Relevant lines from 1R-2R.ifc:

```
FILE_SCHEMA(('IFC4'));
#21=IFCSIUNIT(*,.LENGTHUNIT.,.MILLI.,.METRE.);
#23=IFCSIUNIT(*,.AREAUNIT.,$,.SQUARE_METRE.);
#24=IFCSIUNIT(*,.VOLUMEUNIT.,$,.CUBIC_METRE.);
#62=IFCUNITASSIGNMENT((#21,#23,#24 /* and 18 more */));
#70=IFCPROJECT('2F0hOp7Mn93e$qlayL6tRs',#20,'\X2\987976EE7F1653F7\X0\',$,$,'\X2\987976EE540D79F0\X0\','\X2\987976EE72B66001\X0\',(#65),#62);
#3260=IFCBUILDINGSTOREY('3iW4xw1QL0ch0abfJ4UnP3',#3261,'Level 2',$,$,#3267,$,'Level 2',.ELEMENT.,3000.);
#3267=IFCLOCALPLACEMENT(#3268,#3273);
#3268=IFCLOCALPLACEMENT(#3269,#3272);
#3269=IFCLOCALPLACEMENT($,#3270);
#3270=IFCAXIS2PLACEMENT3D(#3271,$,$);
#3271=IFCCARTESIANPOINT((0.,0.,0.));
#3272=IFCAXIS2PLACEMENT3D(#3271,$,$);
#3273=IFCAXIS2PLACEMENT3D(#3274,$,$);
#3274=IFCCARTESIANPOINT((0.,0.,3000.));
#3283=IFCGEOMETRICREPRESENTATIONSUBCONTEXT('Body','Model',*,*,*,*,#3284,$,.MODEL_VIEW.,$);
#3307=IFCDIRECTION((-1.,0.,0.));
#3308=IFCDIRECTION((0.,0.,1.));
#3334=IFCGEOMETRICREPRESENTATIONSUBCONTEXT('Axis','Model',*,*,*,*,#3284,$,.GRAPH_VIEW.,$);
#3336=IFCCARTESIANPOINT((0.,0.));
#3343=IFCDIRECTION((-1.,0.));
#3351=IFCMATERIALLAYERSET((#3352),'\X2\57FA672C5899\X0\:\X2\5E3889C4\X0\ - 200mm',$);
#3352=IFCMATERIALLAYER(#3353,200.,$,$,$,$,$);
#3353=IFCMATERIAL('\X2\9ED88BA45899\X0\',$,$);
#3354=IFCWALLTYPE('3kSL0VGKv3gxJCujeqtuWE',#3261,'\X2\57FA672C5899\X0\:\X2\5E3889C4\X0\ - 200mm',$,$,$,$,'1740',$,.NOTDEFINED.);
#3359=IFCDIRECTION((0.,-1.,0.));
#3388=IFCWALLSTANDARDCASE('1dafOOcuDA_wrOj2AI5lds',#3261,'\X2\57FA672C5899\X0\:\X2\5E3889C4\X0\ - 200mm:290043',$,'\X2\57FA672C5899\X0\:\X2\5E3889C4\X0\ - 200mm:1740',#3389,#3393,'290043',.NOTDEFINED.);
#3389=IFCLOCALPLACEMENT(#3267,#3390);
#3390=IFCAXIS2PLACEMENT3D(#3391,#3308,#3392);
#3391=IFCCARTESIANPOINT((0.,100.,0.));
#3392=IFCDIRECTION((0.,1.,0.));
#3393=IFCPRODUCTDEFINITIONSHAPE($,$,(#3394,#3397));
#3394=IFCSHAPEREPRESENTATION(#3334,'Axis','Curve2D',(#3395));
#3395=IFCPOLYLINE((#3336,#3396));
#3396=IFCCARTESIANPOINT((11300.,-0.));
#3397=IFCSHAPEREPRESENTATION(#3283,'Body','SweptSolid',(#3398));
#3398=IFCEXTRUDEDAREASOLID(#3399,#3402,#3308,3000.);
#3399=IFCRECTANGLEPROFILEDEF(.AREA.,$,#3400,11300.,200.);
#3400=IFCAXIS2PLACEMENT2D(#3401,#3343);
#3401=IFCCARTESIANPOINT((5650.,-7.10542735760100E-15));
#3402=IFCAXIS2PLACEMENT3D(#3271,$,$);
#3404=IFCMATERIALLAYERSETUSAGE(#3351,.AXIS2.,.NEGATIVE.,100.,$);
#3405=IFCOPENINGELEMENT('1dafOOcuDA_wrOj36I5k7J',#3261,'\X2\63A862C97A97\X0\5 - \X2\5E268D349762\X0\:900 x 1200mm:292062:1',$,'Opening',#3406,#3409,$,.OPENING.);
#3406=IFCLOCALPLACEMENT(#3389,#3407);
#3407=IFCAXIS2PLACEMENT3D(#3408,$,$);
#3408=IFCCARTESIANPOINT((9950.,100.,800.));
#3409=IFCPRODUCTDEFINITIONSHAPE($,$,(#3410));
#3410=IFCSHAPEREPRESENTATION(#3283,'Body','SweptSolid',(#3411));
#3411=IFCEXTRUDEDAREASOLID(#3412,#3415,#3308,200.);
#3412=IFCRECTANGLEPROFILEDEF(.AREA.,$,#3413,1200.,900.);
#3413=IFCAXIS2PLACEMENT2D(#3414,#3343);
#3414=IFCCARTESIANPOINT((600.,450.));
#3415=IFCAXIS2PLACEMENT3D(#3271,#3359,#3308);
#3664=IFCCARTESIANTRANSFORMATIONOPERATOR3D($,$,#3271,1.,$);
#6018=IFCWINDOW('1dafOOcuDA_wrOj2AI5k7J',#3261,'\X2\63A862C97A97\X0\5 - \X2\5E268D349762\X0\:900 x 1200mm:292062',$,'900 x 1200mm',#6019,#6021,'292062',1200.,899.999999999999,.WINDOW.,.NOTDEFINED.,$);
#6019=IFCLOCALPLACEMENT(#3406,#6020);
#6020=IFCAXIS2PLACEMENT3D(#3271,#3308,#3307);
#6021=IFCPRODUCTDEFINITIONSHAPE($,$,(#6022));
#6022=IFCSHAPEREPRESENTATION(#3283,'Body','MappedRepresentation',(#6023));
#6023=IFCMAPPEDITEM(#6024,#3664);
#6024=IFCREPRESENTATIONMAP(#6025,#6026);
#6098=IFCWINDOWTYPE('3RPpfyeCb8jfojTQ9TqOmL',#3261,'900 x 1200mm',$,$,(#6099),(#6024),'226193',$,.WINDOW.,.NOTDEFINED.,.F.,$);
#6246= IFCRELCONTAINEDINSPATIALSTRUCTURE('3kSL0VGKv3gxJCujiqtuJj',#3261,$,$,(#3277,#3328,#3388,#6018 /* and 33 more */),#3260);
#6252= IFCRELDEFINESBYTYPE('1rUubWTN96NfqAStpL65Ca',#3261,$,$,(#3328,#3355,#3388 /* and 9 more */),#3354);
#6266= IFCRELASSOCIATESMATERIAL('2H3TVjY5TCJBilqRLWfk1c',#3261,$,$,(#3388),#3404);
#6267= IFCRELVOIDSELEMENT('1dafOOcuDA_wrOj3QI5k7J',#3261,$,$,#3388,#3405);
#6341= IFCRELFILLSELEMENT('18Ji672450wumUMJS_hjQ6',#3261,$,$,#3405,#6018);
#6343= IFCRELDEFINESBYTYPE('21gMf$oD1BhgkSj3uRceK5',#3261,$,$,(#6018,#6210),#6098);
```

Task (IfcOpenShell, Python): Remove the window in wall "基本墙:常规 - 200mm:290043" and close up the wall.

```python
import ifcopenshell
import ifcopenshell.api.feature
import ifcopenshell.api.root
import ifcopenshell.geom
import ifcopenshell.util.shape

model = ifcopenshell.open("1R-2R.ifc")
settings = ifcopenshell.geom.settings()


def volume(element):
    """Net volume in cubic metres, openings subtracted."""
    shape = ifcopenshell.geom.create_shape(settings, element)
    return ifcopenshell.util.shape.get_volume(shape.geometry)


window = model.by_guid("1dafOOcuDA_wrOj2AI5k7J")
opening = window.FillsVoids[0].RelatingOpeningElement
wall = opening.VoidsElements[0].RelatingBuildingElement
before = volume(wall)

ifcopenshell.api.root.remove_product(model, product=window)
ifcopenshell.api.feature.remove_feature(model, feature=opening)

after = volume(wall)

print(f"wall volume {before:.3f} -> {after:.3f} m3")

model.write("1R-2R_rev.ifc")
```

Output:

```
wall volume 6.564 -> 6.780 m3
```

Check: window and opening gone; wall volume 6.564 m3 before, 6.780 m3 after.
